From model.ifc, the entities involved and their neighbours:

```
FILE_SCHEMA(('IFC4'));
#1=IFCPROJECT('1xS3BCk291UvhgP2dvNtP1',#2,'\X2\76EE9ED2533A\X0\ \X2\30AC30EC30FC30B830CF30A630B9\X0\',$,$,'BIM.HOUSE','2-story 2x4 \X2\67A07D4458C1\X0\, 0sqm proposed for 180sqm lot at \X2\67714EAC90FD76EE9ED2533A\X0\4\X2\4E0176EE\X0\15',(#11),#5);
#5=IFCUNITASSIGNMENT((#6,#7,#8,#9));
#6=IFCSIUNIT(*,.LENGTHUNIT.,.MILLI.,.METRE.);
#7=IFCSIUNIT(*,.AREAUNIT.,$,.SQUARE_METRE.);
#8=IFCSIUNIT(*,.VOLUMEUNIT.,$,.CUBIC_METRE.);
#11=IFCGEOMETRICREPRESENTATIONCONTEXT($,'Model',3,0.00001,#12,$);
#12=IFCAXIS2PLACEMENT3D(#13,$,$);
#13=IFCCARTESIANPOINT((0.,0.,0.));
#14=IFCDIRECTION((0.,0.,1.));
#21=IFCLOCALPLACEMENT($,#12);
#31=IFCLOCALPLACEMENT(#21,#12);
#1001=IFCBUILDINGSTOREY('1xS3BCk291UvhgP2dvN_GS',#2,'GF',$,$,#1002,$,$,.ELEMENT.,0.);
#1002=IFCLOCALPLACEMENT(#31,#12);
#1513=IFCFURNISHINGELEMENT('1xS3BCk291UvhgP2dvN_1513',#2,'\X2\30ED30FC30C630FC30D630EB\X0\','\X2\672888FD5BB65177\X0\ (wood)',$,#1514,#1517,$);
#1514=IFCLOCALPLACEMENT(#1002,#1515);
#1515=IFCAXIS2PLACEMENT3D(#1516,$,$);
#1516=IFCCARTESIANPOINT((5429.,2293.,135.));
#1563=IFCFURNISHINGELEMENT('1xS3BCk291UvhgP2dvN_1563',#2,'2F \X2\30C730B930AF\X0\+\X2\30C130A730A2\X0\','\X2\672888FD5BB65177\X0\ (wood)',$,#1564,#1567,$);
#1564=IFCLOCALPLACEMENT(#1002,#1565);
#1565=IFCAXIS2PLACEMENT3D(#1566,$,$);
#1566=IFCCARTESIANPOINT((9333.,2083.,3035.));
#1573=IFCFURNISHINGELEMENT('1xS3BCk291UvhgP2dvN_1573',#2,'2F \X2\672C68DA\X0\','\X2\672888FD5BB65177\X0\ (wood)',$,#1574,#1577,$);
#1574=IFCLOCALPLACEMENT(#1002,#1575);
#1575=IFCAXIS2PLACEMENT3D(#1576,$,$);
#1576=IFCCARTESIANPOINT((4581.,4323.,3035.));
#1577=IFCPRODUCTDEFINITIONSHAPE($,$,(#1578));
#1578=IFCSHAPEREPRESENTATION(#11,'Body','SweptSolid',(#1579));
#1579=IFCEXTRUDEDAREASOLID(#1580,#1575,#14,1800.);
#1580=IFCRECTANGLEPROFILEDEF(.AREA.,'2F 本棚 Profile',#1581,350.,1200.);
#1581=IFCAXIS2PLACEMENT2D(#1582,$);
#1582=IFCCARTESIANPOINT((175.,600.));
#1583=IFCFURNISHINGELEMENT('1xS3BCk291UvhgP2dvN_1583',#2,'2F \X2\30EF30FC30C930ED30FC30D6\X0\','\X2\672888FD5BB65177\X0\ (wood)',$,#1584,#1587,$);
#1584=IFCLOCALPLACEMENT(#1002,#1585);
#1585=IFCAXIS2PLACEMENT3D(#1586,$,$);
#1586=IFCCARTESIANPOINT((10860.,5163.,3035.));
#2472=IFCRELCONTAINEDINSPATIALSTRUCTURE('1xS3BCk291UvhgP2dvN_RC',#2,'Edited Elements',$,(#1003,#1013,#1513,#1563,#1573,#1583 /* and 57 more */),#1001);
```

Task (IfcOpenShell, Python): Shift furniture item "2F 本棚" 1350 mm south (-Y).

```python
import ifcopenshell
import ifcopenshell.api.geometry
import ifcopenshell.util.placement
import ifcopenshell.util.unit

model = ifcopenshell.open("model.ifc")
unit_scale = ifcopenshell.util.unit.calculate_unit_scale(model)

item = model.by_guid("1xS3BCk291UvhgP2dvN_1573")
matrix = ifcopenshell.util.placement.get_local_placement(item.ObjectPlacement)
matrix[1, 3] -= 1.35 / unit_scale
ifcopenshell.api.geometry.edit_object_placement(model, product=item, matrix=matrix, is_si=False)

print(ifcopenshell.util.placement.get_local_placement(item.ObjectPlacement).round(3) + 0.0)

model.write("model_edited.ifc")
```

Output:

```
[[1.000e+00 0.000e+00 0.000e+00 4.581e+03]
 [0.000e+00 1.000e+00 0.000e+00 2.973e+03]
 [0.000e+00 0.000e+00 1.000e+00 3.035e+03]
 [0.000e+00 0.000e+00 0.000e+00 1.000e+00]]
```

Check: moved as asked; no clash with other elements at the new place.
